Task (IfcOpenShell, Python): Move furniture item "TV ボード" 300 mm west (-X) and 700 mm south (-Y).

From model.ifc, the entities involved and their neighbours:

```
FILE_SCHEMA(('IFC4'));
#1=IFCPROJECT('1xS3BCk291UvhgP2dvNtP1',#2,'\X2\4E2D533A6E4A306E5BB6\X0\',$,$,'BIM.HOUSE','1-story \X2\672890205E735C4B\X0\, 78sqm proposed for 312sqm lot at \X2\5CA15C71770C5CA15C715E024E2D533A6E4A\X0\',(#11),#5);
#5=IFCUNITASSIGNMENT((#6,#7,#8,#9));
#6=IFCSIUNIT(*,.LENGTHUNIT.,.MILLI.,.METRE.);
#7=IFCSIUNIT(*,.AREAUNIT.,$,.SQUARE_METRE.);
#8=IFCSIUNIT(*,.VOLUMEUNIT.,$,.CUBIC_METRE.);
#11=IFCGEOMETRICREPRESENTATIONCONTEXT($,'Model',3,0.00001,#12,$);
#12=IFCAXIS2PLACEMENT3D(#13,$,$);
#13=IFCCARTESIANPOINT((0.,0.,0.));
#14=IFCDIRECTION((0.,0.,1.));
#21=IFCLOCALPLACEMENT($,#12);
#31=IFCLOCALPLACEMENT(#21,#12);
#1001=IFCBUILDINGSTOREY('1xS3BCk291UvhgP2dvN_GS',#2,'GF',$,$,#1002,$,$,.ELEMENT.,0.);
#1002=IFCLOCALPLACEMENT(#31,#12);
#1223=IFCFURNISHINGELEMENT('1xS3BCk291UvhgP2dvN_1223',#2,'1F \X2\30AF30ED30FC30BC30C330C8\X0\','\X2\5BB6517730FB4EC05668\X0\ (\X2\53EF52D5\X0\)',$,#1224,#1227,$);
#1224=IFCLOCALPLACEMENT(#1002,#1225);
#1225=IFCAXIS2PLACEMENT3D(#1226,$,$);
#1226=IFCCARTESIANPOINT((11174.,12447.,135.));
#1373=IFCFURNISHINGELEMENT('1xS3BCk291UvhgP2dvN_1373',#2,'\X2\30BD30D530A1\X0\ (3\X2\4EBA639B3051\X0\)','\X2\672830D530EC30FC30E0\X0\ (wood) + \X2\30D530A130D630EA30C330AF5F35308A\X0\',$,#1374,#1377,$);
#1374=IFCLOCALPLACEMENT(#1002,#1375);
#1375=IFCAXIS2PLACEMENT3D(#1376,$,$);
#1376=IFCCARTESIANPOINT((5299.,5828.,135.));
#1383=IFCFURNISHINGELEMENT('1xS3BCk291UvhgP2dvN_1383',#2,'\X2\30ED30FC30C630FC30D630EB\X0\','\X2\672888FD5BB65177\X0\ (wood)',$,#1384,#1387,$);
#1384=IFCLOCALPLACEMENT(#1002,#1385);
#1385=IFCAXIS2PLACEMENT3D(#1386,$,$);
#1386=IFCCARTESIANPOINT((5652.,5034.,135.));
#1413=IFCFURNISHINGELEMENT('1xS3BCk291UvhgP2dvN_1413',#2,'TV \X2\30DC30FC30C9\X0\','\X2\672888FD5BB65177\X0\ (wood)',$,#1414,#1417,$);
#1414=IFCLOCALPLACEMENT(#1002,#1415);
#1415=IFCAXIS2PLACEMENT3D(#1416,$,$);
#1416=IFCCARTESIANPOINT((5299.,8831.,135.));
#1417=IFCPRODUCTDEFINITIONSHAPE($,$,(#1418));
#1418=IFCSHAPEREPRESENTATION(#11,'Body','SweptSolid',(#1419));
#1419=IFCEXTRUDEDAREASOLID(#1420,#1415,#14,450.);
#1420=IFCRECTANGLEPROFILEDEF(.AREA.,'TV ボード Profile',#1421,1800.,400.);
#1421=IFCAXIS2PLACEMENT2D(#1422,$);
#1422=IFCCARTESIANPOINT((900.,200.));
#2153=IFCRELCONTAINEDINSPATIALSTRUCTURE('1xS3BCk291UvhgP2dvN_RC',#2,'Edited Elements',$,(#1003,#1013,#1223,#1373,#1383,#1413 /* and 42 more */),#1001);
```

```python
import ifcopenshell
import ifcopenshell.api.geometry
import ifcopenshell.util.placement
import ifcopenshell.util.unit

model = ifcopenshell.open("model.ifc")
unit_scale = ifcopenshell.util.unit.calculate_unit_scale(model)

item = model.by_guid("1xS3BCk291UvhgP2dvN_1413")
matrix = ifcopenshell.util.placement.get_local_placement(item.ObjectPlacement)
matrix[0, 3] -= 0.3 / unit_scale
matrix[1, 3] -= 0.7 / unit_scale
ifcopenshell.api.geometry.edit_object_placement(model, product=item, matrix=matrix, is_si=False)

print(ifcopenshell.util.placement.get_local_placement(item.ObjectPlacement).round(3) + 0.0)

model.write("model_updated.ifc")
```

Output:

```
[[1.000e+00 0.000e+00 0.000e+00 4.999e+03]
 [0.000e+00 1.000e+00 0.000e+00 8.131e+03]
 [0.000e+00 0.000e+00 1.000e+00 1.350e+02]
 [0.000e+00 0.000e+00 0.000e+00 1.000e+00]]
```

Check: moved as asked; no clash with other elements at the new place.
